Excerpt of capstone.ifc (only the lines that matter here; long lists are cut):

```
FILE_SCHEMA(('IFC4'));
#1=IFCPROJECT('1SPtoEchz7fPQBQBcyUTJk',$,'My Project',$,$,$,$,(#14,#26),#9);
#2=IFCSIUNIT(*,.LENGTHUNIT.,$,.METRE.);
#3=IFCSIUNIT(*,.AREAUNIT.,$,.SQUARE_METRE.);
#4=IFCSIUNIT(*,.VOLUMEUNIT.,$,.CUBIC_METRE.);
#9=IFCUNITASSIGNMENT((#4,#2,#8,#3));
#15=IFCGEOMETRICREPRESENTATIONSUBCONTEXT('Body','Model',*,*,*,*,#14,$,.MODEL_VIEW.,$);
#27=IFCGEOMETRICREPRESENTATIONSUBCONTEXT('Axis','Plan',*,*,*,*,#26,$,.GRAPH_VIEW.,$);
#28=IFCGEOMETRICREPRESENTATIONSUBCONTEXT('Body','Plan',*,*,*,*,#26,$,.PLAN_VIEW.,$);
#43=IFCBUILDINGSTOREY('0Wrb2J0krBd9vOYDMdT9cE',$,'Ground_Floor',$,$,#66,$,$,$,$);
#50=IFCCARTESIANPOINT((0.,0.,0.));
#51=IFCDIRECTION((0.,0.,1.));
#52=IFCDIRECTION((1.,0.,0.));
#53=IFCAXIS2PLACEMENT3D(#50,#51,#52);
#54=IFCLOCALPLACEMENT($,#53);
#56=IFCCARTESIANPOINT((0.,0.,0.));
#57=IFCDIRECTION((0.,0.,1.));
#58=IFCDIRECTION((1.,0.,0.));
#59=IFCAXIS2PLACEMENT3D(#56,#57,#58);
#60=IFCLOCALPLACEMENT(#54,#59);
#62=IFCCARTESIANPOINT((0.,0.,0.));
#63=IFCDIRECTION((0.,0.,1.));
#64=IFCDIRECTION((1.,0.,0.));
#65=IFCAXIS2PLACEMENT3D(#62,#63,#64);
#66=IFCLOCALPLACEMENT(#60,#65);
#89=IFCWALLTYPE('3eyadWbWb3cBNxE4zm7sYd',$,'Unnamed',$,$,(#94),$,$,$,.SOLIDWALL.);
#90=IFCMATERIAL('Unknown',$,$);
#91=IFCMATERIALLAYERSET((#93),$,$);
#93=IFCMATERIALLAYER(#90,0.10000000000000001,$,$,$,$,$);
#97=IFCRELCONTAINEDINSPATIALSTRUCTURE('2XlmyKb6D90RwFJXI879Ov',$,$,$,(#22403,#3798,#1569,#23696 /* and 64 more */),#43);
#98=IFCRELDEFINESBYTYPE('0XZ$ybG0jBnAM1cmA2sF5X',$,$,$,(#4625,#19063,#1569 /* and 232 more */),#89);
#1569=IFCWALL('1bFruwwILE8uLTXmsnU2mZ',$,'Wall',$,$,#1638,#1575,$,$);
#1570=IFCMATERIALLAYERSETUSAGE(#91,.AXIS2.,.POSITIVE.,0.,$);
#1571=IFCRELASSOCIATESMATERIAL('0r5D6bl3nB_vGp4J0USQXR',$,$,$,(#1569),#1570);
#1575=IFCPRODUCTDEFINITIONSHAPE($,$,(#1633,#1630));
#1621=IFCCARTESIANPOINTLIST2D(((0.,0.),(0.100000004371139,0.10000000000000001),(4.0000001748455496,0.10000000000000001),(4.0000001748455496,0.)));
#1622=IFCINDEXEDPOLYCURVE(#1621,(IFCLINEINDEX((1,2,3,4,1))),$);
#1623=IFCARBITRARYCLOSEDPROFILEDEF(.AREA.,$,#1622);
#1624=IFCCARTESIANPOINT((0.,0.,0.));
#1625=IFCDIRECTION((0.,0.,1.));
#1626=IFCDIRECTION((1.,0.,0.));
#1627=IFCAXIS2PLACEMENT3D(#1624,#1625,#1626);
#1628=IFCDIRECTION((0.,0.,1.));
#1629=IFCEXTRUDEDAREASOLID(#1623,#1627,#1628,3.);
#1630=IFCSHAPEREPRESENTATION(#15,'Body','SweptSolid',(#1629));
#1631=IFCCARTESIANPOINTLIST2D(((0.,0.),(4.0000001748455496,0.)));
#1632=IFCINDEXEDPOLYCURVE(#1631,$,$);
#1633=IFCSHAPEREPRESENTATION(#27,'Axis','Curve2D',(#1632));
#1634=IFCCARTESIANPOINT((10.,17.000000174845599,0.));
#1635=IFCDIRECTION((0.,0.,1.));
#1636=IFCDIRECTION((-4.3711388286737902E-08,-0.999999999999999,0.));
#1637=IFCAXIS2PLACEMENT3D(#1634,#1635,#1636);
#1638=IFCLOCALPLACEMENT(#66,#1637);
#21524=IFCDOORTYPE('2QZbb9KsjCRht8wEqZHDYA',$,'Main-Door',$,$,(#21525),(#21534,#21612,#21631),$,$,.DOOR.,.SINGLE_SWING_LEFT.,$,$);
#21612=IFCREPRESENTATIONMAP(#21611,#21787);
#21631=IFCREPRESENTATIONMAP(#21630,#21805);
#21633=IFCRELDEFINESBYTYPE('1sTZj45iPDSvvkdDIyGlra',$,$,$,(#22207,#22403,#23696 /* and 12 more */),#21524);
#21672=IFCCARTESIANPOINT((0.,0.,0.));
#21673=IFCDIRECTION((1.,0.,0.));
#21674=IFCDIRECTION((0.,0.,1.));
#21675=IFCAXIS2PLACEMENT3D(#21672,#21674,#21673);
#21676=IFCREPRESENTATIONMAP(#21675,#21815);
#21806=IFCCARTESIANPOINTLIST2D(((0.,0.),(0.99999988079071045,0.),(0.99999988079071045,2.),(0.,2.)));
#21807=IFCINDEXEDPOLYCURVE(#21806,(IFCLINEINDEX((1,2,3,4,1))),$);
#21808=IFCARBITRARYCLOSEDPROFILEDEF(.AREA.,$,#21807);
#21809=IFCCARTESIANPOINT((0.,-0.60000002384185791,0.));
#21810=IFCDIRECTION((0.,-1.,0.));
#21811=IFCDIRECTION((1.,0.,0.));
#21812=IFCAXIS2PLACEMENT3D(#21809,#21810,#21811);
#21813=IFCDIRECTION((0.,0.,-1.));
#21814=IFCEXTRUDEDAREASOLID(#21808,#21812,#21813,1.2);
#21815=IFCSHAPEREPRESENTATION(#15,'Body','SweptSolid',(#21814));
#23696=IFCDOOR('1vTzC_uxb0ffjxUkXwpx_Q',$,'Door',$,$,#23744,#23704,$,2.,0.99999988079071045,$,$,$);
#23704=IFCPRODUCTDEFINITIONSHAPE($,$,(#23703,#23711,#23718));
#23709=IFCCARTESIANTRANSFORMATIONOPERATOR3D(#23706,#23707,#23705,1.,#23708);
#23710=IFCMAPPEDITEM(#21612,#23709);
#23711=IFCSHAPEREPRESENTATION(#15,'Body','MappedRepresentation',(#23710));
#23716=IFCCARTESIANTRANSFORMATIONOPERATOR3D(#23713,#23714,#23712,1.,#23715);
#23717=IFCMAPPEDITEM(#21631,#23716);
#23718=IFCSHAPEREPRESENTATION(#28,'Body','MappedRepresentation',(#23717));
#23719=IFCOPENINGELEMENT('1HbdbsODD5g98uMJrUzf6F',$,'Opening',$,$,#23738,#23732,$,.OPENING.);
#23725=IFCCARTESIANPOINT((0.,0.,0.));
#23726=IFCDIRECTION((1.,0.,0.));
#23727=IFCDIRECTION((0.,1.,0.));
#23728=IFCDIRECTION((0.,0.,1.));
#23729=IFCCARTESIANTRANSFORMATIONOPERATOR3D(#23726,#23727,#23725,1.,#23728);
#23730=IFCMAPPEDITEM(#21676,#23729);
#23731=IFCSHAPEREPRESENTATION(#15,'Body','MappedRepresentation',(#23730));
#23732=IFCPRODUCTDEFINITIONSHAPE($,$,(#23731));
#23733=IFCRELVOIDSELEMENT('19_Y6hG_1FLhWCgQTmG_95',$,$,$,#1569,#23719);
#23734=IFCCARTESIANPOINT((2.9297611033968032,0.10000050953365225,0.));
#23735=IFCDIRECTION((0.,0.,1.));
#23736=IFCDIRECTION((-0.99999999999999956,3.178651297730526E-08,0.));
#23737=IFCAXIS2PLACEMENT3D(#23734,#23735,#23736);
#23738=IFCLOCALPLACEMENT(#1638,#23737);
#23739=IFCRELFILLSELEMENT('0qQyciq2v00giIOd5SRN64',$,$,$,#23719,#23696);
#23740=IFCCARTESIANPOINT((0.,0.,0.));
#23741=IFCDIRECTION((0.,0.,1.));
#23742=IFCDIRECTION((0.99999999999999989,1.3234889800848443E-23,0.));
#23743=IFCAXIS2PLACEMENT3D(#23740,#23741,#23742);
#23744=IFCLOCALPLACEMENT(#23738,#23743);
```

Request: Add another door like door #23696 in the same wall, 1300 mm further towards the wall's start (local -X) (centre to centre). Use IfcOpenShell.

```python
import ifcopenshell
import ifcopenshell.api.feature
import ifcopenshell.api.geometry
import ifcopenshell.api.root
import ifcopenshell.geom
import ifcopenshell.util.element
import ifcopenshell.util.placement
import ifcopenshell.util.shape
import ifcopenshell.util.unit

model = ifcopenshell.open("capstone.ifc")
unit_scale = ifcopenshell.util.unit.calculate_unit_scale(model)
settings = ifcopenshell.geom.settings()


def volume(element):
    """Net volume in cubic metres, openings subtracted."""
    shape = ifcopenshell.geom.create_shape(settings, element)
    return ifcopenshell.util.shape.get_volume(shape.geometry)


door = model.by_guid("1vTzC_uxb0ffjxUkXwpx_Q")
opening = door.FillsVoids[0].RelatingOpeningElement
wall = opening.VoidsElements[0].RelatingBuildingElement
before = volume(wall)
shift = ifcopenshell.util.placement.get_local_placement(wall.ObjectPlacement)[:3, 0] * -1.3 / unit_scale

# copy_class copies the void relationship, type, container and properties, but no geometry.
new_opening = ifcopenshell.api.root.copy_class(model, product=opening)
new_opening.Representation = ifcopenshell.util.element.copy_deep(
    model, opening.Representation, exclude=["IfcGeometricRepresentationContext", "IfcRepresentationMap"]
)
new_door = ifcopenshell.api.root.copy_class(model, product=door)
new_door.Representation = ifcopenshell.util.element.copy_deep(
    model, door.Representation, exclude=["IfcGeometricRepresentationContext", "IfcRepresentationMap"]
)
ifcopenshell.api.feature.add_filling(model, opening=new_opening, element=new_door)

for old, new in ((opening, new_opening), (door, new_door)):
    matrix = ifcopenshell.util.placement.get_local_placement(old.ObjectPlacement)
    matrix[:3, 3] += shift
    ifcopenshell.api.geometry.edit_object_placement(model, product=new, matrix=matrix, is_si=False)

after = volume(wall)

print(f"wall volume {before:.3f} -> {after:.3f} m3")

model.write("capstone-out.ifc")
```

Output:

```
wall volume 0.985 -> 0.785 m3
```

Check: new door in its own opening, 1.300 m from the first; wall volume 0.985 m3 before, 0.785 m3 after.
